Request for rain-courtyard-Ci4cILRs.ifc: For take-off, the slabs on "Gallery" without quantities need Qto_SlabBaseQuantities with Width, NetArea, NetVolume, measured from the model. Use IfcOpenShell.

First a look at what the model holds.

```python
import ifcopenshell
import ifcopenshell.util.element
import ifcopenshell.util.unit

model = ifcopenshell.open("rain-courtyard-Ci4cILRs.ifc")
print(model.schema)
for unit_type in ("LENGTHUNIT", "AREAUNIT", "VOLUMEUNIT"):
    print(unit_type, ifcopenshell.util.unit.calculate_unit_scale(model, unit_type))
storey = next(s for s in model.by_type("IfcBuildingStorey") if s.Name == "Gallery")
slabs = [e for e in ifcopenshell.util.element.get_decomposition(storey) if e.is_a("IfcSlab")]
for e in sorted(slabs, key=lambda e: e.id()):
    print(e.id(), e.is_a(), e.Name, list(ifcopenshell.util.element.get_psets(e, qtos_only=True)), sep=" | ")
```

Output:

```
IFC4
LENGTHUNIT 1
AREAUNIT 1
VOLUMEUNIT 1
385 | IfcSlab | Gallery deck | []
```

```python
import ifcopenshell
import ifcopenshell.api.pset
import ifcopenshell.geom
import ifcopenshell.util.element
import ifcopenshell.util.shape
import ifcopenshell.util.unit

model = ifcopenshell.open("rain-courtyard-Ci4cILRs.ifc")
unit_scale = ifcopenshell.util.unit.calculate_unit_scale(model)
area_scale = ifcopenshell.util.unit.calculate_unit_scale(model, "AREAUNIT")
volume_scale = ifcopenshell.util.unit.calculate_unit_scale(model, "VOLUMEUNIT")
settings = ifcopenshell.geom.settings()

storey = next(s for s in model.by_type("IfcBuildingStorey") if s.Name == "Gallery")
slabs = [e for e in ifcopenshell.util.element.get_decomposition(storey) if e.is_a("IfcSlab")]

for e in sorted(slabs, key=lambda e: e.id()):
    if ifcopenshell.util.element.get_psets(e, qtos_only=True, should_inherit=False):
        continue
    # Geometry comes back in metres, in the element's own axes.
    shape = ifcopenshell.geom.create_shape(settings, e)
    values = {
        "Width": ifcopenshell.util.shape.get_z(shape.geometry) / unit_scale,
        "NetArea": ifcopenshell.util.shape.get_footprint_area(shape.geometry) / area_scale,
        "NetVolume": ifcopenshell.util.shape.get_volume(shape.geometry) / volume_scale,
    }
    qto = ifcopenshell.api.pset.add_qto(model, product=e, name="Qto_SlabBaseQuantities")
    ifcopenshell.api.pset.edit_qto(model, qto=qto, properties=values)
    print(e.id(), {k: round(v, 3) for k, v in values.items()})

model.write("rain-courtyard-Ci4cILRs_v2.ifc")
```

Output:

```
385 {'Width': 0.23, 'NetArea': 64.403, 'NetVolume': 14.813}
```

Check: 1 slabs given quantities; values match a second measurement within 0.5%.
